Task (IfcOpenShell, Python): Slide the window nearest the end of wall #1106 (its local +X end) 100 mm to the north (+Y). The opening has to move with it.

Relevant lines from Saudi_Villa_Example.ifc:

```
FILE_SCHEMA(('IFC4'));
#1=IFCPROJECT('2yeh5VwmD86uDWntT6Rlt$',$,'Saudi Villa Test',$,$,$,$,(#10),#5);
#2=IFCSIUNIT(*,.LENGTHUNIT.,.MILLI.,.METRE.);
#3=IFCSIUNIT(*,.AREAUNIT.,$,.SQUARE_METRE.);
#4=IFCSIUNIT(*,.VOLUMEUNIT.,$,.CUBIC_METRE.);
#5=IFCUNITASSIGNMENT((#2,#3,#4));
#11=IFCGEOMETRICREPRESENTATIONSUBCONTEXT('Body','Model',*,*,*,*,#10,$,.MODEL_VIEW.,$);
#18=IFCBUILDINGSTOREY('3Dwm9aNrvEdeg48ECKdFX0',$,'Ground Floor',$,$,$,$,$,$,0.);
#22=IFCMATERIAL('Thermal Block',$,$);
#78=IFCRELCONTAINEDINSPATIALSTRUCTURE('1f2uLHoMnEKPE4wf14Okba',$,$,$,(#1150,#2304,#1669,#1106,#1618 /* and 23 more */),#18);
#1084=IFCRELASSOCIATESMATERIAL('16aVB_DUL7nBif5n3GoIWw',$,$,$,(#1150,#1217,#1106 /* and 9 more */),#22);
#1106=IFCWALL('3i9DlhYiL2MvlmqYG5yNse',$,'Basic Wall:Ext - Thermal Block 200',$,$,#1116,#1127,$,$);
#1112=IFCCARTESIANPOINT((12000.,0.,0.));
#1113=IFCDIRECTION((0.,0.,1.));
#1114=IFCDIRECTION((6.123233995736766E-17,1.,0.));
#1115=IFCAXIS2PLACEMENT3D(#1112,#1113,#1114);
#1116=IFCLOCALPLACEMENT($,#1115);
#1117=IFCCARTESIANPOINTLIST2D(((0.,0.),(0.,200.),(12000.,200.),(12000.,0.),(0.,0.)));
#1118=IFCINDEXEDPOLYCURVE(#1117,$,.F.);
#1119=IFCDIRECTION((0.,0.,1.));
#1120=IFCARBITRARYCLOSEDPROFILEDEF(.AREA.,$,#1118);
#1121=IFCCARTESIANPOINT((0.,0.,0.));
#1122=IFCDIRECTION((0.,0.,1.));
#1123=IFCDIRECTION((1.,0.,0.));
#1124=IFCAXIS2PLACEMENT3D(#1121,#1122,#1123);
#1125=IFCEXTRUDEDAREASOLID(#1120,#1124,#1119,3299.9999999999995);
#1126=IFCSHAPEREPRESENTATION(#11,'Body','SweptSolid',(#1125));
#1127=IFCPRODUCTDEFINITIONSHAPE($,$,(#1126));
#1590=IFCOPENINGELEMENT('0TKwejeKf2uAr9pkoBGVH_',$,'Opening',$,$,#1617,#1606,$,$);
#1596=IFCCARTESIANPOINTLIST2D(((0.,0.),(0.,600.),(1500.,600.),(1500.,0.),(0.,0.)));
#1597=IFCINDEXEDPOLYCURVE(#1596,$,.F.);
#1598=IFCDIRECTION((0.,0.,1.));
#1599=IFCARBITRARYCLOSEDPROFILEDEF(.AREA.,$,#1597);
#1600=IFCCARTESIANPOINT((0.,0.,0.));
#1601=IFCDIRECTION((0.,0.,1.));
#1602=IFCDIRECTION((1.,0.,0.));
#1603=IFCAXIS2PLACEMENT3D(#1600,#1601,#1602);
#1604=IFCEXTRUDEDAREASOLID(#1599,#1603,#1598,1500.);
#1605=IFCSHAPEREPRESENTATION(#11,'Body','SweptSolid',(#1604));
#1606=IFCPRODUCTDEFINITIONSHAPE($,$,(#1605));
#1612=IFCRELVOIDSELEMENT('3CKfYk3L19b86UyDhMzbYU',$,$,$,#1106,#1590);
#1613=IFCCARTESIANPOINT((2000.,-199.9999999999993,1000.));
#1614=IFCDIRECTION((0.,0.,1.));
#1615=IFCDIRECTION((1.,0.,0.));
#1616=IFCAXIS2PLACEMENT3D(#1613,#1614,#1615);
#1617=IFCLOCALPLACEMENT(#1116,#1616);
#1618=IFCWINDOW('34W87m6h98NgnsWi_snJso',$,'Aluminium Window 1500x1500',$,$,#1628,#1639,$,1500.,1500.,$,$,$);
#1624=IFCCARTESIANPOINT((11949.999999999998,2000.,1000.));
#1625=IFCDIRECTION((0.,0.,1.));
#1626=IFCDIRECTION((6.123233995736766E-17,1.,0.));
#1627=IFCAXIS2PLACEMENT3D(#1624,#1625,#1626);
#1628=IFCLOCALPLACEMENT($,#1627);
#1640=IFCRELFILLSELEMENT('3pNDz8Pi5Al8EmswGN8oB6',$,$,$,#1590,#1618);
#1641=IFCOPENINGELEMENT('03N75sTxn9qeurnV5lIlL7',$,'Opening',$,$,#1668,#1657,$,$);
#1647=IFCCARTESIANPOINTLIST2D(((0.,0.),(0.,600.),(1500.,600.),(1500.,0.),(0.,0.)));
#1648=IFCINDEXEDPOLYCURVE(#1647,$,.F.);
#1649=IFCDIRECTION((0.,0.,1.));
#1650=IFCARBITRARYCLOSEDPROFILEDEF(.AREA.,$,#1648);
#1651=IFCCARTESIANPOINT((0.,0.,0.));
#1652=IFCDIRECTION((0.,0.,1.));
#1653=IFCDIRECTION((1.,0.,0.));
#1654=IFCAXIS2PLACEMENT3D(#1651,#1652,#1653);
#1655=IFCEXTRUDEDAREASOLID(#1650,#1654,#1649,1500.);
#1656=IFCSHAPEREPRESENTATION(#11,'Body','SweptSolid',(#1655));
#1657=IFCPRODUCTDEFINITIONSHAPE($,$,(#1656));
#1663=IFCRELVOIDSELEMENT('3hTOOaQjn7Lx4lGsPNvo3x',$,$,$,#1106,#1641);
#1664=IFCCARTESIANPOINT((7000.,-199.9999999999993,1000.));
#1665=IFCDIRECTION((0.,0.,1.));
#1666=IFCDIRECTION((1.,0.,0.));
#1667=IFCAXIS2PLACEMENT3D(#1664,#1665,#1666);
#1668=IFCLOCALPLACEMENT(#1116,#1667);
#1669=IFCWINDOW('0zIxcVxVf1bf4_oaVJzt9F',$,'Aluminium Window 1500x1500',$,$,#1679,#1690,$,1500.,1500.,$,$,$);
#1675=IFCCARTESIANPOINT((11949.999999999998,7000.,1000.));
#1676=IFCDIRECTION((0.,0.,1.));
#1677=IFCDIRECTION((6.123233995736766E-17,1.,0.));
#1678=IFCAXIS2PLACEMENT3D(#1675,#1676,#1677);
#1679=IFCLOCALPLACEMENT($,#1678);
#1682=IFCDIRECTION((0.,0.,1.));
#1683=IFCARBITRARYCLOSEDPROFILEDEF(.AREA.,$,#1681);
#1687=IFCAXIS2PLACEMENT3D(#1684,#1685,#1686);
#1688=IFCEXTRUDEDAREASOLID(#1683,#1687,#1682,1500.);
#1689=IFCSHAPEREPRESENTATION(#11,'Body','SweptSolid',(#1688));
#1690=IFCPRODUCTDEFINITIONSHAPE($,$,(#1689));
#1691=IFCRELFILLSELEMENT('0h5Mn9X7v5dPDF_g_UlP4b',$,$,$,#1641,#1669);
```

```python
import ifcopenshell
import ifcopenshell.api.geometry
import ifcopenshell.util.placement

model = ifcopenshell.open("Saudi_Villa_Example.ifc")

window = model.by_guid("0zIxcVxVf1bf4_oaVJzt9F")
opening = window.FillsVoids[0].RelatingOpeningElement
wall = opening.VoidsElements[0].RelatingBuildingElement

wall_matrix = ifcopenshell.util.placement.get_local_placement(wall.ObjectPlacement)
shift = wall_matrix[:3, 0] * 100.0
before = ifcopenshell.util.placement.get_local_placement(window.ObjectPlacement)[:3, 3].copy()

# The window is not placed relative to its opening, so move both.
for product in (opening, window):
    matrix = ifcopenshell.util.placement.get_local_placement(product.ObjectPlacement)
    matrix[:3, 3] += shift
    ifcopenshell.api.geometry.edit_object_placement(model, product=product, matrix=matrix, is_si=False)

after = ifcopenshell.util.placement.get_local_placement(window.ObjectPlacement)[:3, 3]
print("window moved by", (after - before).round(3) + 0.0)

model.write("Saudi_Villa_Example_updated.ifc")
```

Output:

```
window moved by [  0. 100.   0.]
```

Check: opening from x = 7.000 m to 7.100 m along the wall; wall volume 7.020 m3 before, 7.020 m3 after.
